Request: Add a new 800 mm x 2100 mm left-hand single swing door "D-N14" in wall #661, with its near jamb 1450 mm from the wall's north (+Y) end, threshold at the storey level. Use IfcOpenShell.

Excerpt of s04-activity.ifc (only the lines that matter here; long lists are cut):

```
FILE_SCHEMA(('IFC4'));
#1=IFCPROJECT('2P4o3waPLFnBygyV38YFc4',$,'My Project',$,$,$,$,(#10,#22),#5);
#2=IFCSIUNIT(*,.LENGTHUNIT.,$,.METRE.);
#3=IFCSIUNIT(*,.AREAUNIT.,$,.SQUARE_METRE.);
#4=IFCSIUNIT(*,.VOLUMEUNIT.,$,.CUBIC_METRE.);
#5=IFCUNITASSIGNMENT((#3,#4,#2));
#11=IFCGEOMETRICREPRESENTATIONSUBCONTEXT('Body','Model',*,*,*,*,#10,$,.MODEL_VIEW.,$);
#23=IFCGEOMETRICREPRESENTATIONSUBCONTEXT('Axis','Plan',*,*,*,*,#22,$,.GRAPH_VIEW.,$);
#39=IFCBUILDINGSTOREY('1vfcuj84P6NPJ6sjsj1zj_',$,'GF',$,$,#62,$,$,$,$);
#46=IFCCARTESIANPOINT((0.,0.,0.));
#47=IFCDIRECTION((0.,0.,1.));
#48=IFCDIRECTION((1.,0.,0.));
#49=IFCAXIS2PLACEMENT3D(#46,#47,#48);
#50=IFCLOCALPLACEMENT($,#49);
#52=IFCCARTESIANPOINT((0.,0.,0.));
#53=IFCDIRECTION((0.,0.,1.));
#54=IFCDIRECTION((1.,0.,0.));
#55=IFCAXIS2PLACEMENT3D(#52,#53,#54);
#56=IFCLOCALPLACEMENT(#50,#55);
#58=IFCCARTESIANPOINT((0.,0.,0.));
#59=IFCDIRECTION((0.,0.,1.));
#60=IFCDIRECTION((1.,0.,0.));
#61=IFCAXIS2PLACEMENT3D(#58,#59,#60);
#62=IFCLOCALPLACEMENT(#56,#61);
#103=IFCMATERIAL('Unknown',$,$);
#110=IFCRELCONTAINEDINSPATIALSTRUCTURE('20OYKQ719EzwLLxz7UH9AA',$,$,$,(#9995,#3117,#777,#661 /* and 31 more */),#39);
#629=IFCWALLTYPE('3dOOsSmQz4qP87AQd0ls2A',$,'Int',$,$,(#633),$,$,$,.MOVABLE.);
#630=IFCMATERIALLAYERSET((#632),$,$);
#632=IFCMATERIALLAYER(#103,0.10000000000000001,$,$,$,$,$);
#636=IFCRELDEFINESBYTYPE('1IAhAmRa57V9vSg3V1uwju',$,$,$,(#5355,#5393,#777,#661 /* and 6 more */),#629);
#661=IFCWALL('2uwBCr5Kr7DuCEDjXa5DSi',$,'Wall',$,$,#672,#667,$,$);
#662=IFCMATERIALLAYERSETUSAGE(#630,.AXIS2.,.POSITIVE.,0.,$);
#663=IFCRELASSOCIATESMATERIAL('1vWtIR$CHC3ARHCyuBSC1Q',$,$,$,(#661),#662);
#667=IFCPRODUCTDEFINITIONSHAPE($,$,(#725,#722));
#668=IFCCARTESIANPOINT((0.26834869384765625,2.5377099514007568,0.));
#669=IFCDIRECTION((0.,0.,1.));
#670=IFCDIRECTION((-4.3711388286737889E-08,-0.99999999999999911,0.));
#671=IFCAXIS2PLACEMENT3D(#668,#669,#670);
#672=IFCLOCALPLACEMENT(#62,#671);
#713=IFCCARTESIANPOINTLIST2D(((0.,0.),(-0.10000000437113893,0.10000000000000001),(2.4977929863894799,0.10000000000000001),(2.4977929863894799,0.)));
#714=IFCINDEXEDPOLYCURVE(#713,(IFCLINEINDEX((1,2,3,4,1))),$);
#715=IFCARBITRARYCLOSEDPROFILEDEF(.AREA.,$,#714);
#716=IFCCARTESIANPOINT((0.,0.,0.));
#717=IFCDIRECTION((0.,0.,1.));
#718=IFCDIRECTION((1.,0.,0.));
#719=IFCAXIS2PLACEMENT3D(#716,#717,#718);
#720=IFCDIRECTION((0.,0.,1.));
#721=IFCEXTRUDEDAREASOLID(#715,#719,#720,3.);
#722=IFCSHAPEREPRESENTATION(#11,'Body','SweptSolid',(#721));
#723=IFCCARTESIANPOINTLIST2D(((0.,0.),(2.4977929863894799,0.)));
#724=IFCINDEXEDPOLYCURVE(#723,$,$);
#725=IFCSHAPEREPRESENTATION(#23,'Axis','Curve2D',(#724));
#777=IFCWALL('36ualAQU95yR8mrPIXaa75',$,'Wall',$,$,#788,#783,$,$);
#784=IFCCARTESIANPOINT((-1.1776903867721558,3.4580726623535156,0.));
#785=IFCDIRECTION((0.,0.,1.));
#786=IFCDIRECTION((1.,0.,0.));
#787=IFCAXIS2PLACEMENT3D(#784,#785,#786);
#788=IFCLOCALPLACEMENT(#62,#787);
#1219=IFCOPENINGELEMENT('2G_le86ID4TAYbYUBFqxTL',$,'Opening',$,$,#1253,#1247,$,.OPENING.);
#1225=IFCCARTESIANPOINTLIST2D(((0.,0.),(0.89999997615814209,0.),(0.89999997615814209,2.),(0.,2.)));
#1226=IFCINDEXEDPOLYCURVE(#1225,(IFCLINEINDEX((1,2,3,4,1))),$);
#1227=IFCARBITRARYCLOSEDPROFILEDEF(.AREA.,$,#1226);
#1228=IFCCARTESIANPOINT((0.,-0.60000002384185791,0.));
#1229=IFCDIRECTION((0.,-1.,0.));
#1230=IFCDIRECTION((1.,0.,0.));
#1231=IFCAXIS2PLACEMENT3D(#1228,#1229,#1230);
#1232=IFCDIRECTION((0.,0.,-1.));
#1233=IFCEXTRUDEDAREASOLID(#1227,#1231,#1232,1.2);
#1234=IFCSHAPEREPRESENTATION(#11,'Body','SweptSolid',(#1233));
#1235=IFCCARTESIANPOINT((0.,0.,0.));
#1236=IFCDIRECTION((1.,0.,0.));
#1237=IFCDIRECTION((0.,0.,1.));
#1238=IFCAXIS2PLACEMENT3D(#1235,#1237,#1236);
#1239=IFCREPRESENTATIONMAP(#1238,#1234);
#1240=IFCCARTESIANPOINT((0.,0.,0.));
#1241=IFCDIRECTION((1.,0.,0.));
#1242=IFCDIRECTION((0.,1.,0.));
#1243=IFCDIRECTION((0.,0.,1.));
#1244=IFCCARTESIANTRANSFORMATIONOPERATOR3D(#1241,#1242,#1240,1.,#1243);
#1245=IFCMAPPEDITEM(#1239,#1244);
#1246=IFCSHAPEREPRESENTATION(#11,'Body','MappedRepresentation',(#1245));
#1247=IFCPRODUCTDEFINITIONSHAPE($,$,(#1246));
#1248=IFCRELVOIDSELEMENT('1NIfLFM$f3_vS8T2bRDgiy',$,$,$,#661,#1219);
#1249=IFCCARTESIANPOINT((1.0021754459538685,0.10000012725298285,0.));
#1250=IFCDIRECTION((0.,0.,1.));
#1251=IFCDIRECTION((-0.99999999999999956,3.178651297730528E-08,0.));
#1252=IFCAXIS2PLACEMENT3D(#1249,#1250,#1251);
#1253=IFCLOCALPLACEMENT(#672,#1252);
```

```python
import numpy as np
import ifcopenshell
import ifcopenshell.api.feature
import ifcopenshell.api.geometry
import ifcopenshell.api.root
import ifcopenshell.api.spatial
import ifcopenshell.geom
import ifcopenshell.util.element
import ifcopenshell.util.placement
import ifcopenshell.util.representation
import ifcopenshell.util.shape
import ifcopenshell.util.unit

model = ifcopenshell.open("s04-activity.ifc")
unit_scale = ifcopenshell.util.unit.calculate_unit_scale(model)
settings = ifcopenshell.geom.settings()


def volume(element):
    """Net volume in cubic metres, openings subtracted."""
    shape = ifcopenshell.geom.create_shape(settings, element)
    return ifcopenshell.util.shape.get_volume(shape.geometry)


wall = model.by_guid("2uwBCr5Kr7DuCEDjXa5DSi")
storey = ifcopenshell.util.element.get_container(wall, ifc_class="IfcBuildingStorey")
context = ifcopenshell.util.representation.get_context(model, "Model", "Body", "MODEL_VIEW")
before = volume(wall)

width, height, from_end, sill = 0.8, 2.1, 1.45, 0.0  # metres

# The wall runs along its own X axis, and the end named is its -X end.
wall_shape = ifcopenshell.geom.create_shape(settings, wall)
x, y, z = ifcopenshell.util.shape.get_vertices(wall_shape.geometry).T
start = x.min() + from_end
face, thickness = float(y.min()), float(y.max() - y.min())
wall_matrix = ifcopenshell.util.placement.get_local_placement(wall.ObjectPlacement)
level = ifcopenshell.util.placement.get_local_placement(storey.ObjectPlacement)[2, 3]


def in_wall(x, y):
    """Placement at x, y metres in the wall's axes, at sill height."""
    matrix = wall_matrix.copy()
    matrix[:, 3] = wall_matrix @ np.array([x / unit_scale, y / unit_scale, 0.0, 1.0])
    matrix[2, 3] = level + sill / unit_scale
    return matrix


# Opening: a box that overshoots both wall faces by 50 mm.
opening = ifcopenshell.api.root.create_entity(model, ifc_class="IfcOpeningElement", predefined_type="OPENING")
box = ifcopenshell.api.geometry.add_wall_representation(
    model, context=context, length=width, height=height, thickness=thickness + 0.1
)
ifcopenshell.api.geometry.assign_representation(model, product=opening, representation=box)
ifcopenshell.api.geometry.edit_object_placement(model, product=opening, matrix=in_wall(start, face - 0.05), is_si=False)
ifcopenshell.api.feature.add_feature(model, feature=opening, element=wall)

door = ifcopenshell.api.root.create_entity(model, ifc_class="IfcDoor", name="D-N14", predefined_type="DOOR")
door.OverallWidth, door.OverallHeight = width / unit_scale, height / unit_scale
door.OperationType = "SINGLE_SWING_LEFT"
body = ifcopenshell.api.geometry.add_door_representation(
    model,
    context=context,
    overall_width=door.OverallWidth,
    overall_height=door.OverallHeight,
    operation_type="SINGLE_SWING_LEFT",
    lining_properties={"LiningDepth": thickness / unit_scale, "ThresholdDepth": thickness / unit_scale},
)
ifcopenshell.api.geometry.assign_representation(model, product=door, representation=body)
ifcopenshell.api.spatial.assign_container(model, products=[door], relating_structure=storey)
ifcopenshell.api.feature.add_filling(model, opening=opening, element=door)

# The lining spans the wall, so the door starts at the wall face.
ifcopenshell.api.geometry.edit_object_placement(model, product=door, matrix=in_wall(start, face), is_si=False)

after = volume(wall)

print(f"wall volume {before:.3f} -> {after:.3f} m3")

model.write("s04-activity_v2.ifc")
```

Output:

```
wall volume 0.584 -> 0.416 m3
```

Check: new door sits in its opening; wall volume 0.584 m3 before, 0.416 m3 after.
